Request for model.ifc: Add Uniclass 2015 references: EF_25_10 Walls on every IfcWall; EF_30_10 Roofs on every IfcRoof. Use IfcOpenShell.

First a look at what the model holds.

```python
import ifcopenshell

model = ifcopenshell.open("model.ifc")
print(model.schema)
print("classifications:", [c.Name for c in model.by_type("IfcClassification")])
for ifc_class in ("IfcDoor", "IfcRoof", "IfcStair", "IfcWall", "IfcWindow"):
    print(ifc_class, len(model.by_type(ifc_class)))
```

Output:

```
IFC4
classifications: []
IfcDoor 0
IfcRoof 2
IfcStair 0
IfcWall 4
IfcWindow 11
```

```python
import ifcopenshell
import ifcopenshell.api.classification

model = ifcopenshell.open("model.ifc")

system = ifcopenshell.api.classification.add_classification(model, classification="Uniclass 2015")

codes = {
    "IfcWall": ("EF_25_10", "Walls"),
    "IfcRoof": ("EF_30_10", "Roofs"),
}
for ifc_class, (code, name) in codes.items():
    products = model.by_type(ifc_class)
    ifcopenshell.api.classification.add_reference(
        model, products=products, classification=system, identification=code, name=name
    )
    print(code, len(products))

model.write("model_updated.ifc")
```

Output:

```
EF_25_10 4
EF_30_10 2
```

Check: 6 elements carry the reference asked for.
